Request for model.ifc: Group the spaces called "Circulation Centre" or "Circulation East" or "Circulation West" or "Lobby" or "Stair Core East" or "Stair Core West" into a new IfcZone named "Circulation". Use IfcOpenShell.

First a look at what the model holds.

```python
import ifcopenshell

model = ifcopenshell.open("model.ifc")
print(model.schema)
seen = {}
for space in model.by_type("IfcSpace"):
    seen[space.LongName] = seen.get(space.LongName, 0) + 1
for name, count in sorted(seen.items(), key=str):
    print(count, "x", name)
print("zones:", [z.Name for z in model.by_type("IfcZone")][:20])
```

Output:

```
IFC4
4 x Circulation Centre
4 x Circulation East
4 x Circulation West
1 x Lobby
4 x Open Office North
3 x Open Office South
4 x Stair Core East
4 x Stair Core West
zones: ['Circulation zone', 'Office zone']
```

```python
import ifcopenshell
import ifcopenshell.api.group
import ifcopenshell.api.root

model = ifcopenshell.open("model.ifc")

names = {"Circulation Centre", "Circulation East", "Circulation West", "Lobby", "Stair Core East", "Stair Core West"}
spaces = [s for s in model.by_type("IfcSpace") if s.LongName in names]

zone = ifcopenshell.api.root.create_entity(model, ifc_class="IfcZone", name="Circulation")
ifcopenshell.api.group.assign_group(model, products=spaces, group=zone)
print(len(spaces), "spaces in", zone.Name)

model.write("model_edited.ifc")
```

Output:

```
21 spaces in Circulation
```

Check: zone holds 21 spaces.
